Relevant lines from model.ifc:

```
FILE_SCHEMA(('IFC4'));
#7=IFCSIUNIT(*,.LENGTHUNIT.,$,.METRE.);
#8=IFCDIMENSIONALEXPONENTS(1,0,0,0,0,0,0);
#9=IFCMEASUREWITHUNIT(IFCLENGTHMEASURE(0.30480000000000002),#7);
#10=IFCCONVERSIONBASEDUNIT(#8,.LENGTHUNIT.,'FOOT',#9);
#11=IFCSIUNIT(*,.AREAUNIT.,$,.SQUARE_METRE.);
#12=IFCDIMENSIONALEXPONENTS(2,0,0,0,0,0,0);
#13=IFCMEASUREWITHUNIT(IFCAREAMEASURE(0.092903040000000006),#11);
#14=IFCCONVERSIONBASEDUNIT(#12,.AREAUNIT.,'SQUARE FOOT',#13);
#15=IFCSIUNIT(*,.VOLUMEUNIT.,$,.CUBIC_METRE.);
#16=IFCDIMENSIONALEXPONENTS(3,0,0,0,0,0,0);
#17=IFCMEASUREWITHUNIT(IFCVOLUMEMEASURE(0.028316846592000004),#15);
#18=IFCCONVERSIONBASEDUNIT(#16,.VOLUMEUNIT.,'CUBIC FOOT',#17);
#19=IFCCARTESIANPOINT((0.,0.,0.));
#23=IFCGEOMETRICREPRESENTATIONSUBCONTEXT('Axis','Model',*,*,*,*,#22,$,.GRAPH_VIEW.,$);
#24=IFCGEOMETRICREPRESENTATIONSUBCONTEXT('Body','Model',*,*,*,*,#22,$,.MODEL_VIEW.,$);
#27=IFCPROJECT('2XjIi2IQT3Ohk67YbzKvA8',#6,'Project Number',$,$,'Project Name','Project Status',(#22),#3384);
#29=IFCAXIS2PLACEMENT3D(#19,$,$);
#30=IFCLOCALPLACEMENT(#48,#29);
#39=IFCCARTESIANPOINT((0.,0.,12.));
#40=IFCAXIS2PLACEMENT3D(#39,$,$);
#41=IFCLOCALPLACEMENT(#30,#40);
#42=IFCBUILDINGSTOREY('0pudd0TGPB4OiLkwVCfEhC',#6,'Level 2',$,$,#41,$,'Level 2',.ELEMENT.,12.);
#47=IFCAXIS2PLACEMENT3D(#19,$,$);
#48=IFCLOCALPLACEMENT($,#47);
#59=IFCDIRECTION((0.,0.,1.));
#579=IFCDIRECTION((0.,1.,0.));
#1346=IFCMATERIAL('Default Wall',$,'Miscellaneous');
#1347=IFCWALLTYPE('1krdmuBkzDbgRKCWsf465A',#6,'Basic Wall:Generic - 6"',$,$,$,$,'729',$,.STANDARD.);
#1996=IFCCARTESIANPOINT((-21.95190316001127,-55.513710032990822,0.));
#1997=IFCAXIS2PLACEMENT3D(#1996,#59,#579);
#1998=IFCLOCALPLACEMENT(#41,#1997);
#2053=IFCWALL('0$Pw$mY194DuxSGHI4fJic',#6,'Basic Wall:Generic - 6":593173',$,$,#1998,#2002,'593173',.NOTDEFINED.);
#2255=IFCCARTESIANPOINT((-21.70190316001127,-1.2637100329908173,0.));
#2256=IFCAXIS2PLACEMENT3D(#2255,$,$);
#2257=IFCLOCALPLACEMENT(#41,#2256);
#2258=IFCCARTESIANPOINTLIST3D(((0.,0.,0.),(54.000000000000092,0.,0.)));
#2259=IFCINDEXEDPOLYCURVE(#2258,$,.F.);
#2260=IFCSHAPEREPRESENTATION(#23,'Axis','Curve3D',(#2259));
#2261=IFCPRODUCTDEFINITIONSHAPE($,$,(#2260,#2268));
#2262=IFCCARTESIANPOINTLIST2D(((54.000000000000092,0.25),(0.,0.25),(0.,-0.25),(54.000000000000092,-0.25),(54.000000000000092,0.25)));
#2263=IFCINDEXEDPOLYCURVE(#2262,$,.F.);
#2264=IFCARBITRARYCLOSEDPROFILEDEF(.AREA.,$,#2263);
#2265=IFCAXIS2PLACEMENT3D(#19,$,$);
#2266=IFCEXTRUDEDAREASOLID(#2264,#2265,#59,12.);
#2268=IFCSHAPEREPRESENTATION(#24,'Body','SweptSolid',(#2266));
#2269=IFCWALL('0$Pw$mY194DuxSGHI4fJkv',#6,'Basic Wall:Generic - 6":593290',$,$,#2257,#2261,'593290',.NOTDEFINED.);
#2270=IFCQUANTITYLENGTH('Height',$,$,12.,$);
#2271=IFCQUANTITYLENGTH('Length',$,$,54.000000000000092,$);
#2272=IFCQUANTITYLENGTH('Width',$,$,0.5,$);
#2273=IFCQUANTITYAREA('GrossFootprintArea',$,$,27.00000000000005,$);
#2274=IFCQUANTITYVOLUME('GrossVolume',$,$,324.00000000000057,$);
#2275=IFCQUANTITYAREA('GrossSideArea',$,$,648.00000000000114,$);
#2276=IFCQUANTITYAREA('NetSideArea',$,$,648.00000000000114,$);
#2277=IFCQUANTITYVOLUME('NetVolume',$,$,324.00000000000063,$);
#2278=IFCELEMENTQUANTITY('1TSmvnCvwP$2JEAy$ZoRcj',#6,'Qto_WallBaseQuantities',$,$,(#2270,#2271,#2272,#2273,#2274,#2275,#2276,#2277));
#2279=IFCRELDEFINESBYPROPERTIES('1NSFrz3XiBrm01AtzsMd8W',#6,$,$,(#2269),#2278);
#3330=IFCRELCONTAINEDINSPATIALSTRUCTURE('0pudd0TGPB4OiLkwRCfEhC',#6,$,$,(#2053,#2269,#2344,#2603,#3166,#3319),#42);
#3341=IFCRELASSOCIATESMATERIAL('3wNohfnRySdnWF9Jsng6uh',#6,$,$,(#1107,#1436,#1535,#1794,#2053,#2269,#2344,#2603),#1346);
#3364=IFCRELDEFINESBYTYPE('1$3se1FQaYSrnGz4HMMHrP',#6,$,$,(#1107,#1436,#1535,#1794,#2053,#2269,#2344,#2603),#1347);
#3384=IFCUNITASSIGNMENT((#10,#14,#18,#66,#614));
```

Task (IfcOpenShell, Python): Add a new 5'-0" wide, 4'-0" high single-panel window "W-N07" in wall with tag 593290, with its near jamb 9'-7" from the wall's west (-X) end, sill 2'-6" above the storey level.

```python
import numpy as np
import ifcopenshell
import ifcopenshell.api.feature
import ifcopenshell.api.geometry
import ifcopenshell.api.pset
import ifcopenshell.api.root
import ifcopenshell.api.spatial
import ifcopenshell.geom
import ifcopenshell.util.element
import ifcopenshell.util.placement
import ifcopenshell.util.representation
import ifcopenshell.util.shape
import ifcopenshell.util.unit

model = ifcopenshell.open("model.ifc")
unit_scale = ifcopenshell.util.unit.calculate_unit_scale(model)
area_scale = ifcopenshell.util.unit.calculate_unit_scale(model, "AREAUNIT")
volume_scale = ifcopenshell.util.unit.calculate_unit_scale(model, "VOLUMEUNIT")
settings = ifcopenshell.geom.settings()


def volume(element):
    """Net volume in cubic metres, openings subtracted."""
    shape = ifcopenshell.geom.create_shape(settings, element)
    return ifcopenshell.util.shape.get_volume(shape.geometry)


wall = model.by_id(2269)
storey = ifcopenshell.util.element.get_container(wall, ifc_class="IfcBuildingStorey")
context = ifcopenshell.util.representation.get_context(model, "Model", "Body", "MODEL_VIEW")
before = volume(wall)

width, height, from_end, sill = 1.524, 1.2192, 2.921, 0.762  # metres

# The wall runs along its own X axis, and the end named is its -X end.
wall_shape = ifcopenshell.geom.create_shape(settings, wall)
x, y, z = ifcopenshell.util.shape.get_vertices(wall_shape.geometry).T
start = x.min() + from_end
face, thickness = float(y.min()), float(y.max() - y.min())
wall_matrix = ifcopenshell.util.placement.get_local_placement(wall.ObjectPlacement)
level = ifcopenshell.util.placement.get_local_placement(storey.ObjectPlacement)[2, 3]


def in_wall(x, y):
    """Placement at x, y metres in the wall's axes, at sill height."""
    matrix = wall_matrix.copy()
    matrix[:, 3] = wall_matrix @ np.array([x / unit_scale, y / unit_scale, 0.0, 1.0])
    matrix[2, 3] = level + sill / unit_scale
    return matrix


# Opening: a box that overshoots both wall faces by 50 mm.
opening = ifcopenshell.api.root.create_entity(model, ifc_class="IfcOpeningElement", predefined_type="OPENING")
box = ifcopenshell.api.geometry.add_wall_representation(
    model, context=context, length=width, height=height, thickness=thickness + 0.1
)
ifcopenshell.api.geometry.assign_representation(model, product=opening, representation=box)
ifcopenshell.api.geometry.edit_object_placement(model, product=opening, matrix=in_wall(start, face - 0.05), is_si=False)
ifcopenshell.api.feature.add_feature(model, feature=opening, element=wall)

window = ifcopenshell.api.root.create_entity(model, ifc_class="IfcWindow", name="W-N07", predefined_type="WINDOW")
window.OverallWidth, window.OverallHeight = width / unit_scale, height / unit_scale
window.PartitioningType = "SINGLE_PANEL"
body = ifcopenshell.api.geometry.add_window_representation(
    model,
    context=context,
    overall_width=window.OverallWidth,
    overall_height=window.OverallHeight,
    partition_type="SINGLE_PANEL",
)
ifcopenshell.api.geometry.assign_representation(model, product=window, representation=body)
ifcopenshell.api.spatial.assign_container(model, products=[window], relating_structure=storey)
ifcopenshell.api.feature.add_filling(model, opening=opening, element=window)

# Centre the window in the wall's thickness.
ifcopenshell.api.geometry.edit_object_placement(model, product=window, matrix=in_wall(start, face), is_si=False)
window_shape = ifcopenshell.geom.create_shape(settings, window)
depth = ifcopenshell.util.shape.get_vertices(window_shape.geometry)[:, 1]
offset = face + thickness / 2 - (depth.min() + depth.max()) / 2
ifcopenshell.api.geometry.edit_object_placement(model, product=window, matrix=in_wall(start, offset), is_si=False)

after = volume(wall)

# Update the wall's stored quantities.
qto = model.by_id(ifcopenshell.util.element.get_pset(wall, "Qto_WallBaseQuantities", should_inherit=False)["id"])
ifcopenshell.api.pset.edit_qto(model, qto=qto, properties={
    "NetSideArea": after / thickness / area_scale,
    "NetVolume": after / volume_scale,
})

print(f"wall volume {before:.3f} -> {after:.3f} m3")

model.write("model_edited.ifc")
```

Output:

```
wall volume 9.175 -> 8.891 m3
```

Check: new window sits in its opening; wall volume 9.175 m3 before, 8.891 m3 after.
